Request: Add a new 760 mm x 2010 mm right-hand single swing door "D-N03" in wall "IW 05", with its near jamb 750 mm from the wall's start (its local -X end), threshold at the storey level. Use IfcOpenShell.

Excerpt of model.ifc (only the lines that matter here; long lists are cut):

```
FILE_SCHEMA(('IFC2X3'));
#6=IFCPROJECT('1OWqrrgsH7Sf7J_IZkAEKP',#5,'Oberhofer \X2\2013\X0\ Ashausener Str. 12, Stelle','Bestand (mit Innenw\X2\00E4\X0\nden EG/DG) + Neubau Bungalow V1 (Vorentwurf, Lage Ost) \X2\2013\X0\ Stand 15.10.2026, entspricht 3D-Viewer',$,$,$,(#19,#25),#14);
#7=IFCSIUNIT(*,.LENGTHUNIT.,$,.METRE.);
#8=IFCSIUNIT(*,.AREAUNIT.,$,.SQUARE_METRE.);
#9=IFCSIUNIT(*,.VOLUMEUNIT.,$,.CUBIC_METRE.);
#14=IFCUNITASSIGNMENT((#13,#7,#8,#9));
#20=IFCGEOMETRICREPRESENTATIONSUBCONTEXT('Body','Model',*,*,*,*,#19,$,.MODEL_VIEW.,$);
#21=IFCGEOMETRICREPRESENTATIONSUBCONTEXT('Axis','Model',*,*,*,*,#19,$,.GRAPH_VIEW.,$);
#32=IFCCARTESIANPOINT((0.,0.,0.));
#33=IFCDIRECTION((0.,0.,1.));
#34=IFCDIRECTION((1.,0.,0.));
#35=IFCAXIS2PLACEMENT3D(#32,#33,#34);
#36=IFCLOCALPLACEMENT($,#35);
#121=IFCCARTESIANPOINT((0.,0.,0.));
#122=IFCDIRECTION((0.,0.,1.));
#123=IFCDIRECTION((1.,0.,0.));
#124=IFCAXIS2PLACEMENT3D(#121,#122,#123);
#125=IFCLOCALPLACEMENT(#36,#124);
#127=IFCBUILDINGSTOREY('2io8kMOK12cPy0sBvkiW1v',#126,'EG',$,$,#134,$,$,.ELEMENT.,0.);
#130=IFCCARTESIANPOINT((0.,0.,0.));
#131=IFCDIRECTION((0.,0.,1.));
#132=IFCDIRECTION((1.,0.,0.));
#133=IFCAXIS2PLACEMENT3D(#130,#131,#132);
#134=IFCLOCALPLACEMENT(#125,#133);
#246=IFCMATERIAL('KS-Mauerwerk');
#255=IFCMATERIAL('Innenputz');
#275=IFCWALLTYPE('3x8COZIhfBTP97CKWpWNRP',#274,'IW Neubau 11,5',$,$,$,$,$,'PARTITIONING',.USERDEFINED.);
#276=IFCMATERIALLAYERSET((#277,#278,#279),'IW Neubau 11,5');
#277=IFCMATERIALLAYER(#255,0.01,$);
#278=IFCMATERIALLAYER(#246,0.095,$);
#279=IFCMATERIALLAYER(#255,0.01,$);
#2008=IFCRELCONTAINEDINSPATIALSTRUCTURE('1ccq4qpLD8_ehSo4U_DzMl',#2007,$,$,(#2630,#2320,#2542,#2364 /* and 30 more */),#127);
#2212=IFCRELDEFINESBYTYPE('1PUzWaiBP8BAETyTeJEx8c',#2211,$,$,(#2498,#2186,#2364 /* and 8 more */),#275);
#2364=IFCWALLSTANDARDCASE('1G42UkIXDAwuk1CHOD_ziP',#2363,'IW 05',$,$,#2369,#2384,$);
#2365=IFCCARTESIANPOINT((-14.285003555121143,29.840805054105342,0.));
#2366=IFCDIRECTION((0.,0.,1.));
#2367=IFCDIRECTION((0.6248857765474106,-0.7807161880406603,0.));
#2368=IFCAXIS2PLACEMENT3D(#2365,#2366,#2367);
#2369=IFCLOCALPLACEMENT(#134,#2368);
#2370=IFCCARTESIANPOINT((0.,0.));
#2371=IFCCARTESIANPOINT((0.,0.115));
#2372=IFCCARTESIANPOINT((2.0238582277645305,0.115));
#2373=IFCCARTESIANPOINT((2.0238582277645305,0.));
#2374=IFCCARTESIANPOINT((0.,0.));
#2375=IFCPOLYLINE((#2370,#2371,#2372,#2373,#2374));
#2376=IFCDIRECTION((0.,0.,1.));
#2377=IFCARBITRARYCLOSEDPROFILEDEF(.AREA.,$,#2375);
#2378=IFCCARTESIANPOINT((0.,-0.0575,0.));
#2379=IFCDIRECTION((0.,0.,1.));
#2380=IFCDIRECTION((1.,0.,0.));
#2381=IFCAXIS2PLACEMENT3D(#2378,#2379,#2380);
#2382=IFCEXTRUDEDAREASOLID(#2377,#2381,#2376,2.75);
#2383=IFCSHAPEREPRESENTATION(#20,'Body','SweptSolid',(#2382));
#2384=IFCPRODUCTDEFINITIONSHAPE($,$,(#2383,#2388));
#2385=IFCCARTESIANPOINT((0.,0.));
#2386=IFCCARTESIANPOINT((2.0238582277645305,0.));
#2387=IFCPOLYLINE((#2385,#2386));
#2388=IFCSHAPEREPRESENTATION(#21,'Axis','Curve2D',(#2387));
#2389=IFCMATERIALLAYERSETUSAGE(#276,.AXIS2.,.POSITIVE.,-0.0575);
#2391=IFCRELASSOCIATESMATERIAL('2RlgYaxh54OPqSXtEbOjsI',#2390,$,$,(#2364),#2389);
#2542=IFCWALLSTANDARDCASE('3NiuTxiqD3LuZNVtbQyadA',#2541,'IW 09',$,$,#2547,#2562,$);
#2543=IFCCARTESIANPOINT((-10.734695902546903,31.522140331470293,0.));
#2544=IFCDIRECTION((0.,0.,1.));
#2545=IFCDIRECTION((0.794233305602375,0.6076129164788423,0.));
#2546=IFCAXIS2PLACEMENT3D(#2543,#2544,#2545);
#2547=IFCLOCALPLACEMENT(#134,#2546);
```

```python
import numpy as np
import ifcopenshell
import ifcopenshell.api.feature
import ifcopenshell.api.geometry
import ifcopenshell.api.root
import ifcopenshell.api.spatial
import ifcopenshell.api.type
import ifcopenshell.geom
import ifcopenshell.util.element
import ifcopenshell.util.placement
import ifcopenshell.util.representation
import ifcopenshell.util.shape
import ifcopenshell.util.unit

model = ifcopenshell.open("model.ifc")
unit_scale = ifcopenshell.util.unit.calculate_unit_scale(model)
settings = ifcopenshell.geom.settings()


def volume(element):
    """Net volume in cubic metres, openings subtracted."""
    shape = ifcopenshell.geom.create_shape(settings, element)
    return ifcopenshell.util.shape.get_volume(shape.geometry)


wall = model.by_id(2364)
storey = ifcopenshell.util.element.get_container(wall, ifc_class="IfcBuildingStorey")
context = ifcopenshell.util.representation.get_context(model, "Model", "Body", "MODEL_VIEW")
before = volume(wall)

width, height, from_end, sill = 0.76, 2.01, 0.75, 0.0  # metres

# The wall runs along its own X axis, and the end named is its -X end.
wall_shape = ifcopenshell.geom.create_shape(settings, wall)
x, y, z = ifcopenshell.util.shape.get_vertices(wall_shape.geometry).T
start = x.min() + from_end
face, thickness = float(y.min()), float(y.max() - y.min())
wall_matrix = ifcopenshell.util.placement.get_local_placement(wall.ObjectPlacement)
level = ifcopenshell.util.placement.get_local_placement(storey.ObjectPlacement)[2, 3]


def in_wall(x, y):
    """Placement at x, y metres in the wall's axes, at sill height."""
    matrix = wall_matrix.copy()
    matrix[:, 3] = wall_matrix @ np.array([x / unit_scale, y / unit_scale, 0.0, 1.0])
    matrix[2, 3] = level + sill / unit_scale
    return matrix


# Opening: a box that overshoots both wall faces by 50 mm.
opening = ifcopenshell.api.root.create_entity(model, ifc_class="IfcOpeningElement")
box = ifcopenshell.api.geometry.add_wall_representation(
    model, context=context, length=width, height=height, thickness=thickness + 0.1
)
ifcopenshell.api.geometry.assign_representation(model, product=opening, representation=box)
ifcopenshell.api.geometry.edit_object_placement(model, product=opening, matrix=in_wall(start, face - 0.05), is_si=False)
ifcopenshell.api.feature.add_feature(model, feature=opening, element=wall)

door = ifcopenshell.api.root.create_entity(model, ifc_class="IfcDoor", name="D-N03")
door.OverallWidth, door.OverallHeight = width / unit_scale, height / unit_scale
body = ifcopenshell.api.geometry.add_door_representation(
    model,
    context=context,
    overall_width=door.OverallWidth,
    overall_height=door.OverallHeight,
    operation_type="SINGLE_SWING_RIGHT",
    lining_properties={"LiningDepth": thickness / unit_scale, "ThresholdDepth": thickness / unit_scale},
)
ifcopenshell.api.geometry.assign_representation(model, product=door, representation=body)
ifcopenshell.api.spatial.assign_container(model, products=[door], relating_structure=storey)
fills = ifcopenshell.api.feature.add_filling(model, opening=opening, element=door)
fills.OwnerHistory = door.OwnerHistory  # required in IFC2X3

# IFC2X3 keeps the operation on the door style.
style = ifcopenshell.api.root.create_entity(model, ifc_class="IfcDoorStyle", name="D-N03")
style.OperationType, style.ConstructionType = "SINGLE_SWING_RIGHT", "NOTDEFINED"
style.ParameterTakesPrecedence = style.Sizeable = False
ifcopenshell.api.type.assign_type(model, related_objects=[door], relating_type=style)

# The lining spans the wall, so the door starts at the wall face.
ifcopenshell.api.geometry.edit_object_placement(model, product=door, matrix=in_wall(start, face), is_si=False)

after = volume(wall)

print(f"wall volume {before:.3f} -> {after:.3f} m3")

model.write("model_updated.ifc")
```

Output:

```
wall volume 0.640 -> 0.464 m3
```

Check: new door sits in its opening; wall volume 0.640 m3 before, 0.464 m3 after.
